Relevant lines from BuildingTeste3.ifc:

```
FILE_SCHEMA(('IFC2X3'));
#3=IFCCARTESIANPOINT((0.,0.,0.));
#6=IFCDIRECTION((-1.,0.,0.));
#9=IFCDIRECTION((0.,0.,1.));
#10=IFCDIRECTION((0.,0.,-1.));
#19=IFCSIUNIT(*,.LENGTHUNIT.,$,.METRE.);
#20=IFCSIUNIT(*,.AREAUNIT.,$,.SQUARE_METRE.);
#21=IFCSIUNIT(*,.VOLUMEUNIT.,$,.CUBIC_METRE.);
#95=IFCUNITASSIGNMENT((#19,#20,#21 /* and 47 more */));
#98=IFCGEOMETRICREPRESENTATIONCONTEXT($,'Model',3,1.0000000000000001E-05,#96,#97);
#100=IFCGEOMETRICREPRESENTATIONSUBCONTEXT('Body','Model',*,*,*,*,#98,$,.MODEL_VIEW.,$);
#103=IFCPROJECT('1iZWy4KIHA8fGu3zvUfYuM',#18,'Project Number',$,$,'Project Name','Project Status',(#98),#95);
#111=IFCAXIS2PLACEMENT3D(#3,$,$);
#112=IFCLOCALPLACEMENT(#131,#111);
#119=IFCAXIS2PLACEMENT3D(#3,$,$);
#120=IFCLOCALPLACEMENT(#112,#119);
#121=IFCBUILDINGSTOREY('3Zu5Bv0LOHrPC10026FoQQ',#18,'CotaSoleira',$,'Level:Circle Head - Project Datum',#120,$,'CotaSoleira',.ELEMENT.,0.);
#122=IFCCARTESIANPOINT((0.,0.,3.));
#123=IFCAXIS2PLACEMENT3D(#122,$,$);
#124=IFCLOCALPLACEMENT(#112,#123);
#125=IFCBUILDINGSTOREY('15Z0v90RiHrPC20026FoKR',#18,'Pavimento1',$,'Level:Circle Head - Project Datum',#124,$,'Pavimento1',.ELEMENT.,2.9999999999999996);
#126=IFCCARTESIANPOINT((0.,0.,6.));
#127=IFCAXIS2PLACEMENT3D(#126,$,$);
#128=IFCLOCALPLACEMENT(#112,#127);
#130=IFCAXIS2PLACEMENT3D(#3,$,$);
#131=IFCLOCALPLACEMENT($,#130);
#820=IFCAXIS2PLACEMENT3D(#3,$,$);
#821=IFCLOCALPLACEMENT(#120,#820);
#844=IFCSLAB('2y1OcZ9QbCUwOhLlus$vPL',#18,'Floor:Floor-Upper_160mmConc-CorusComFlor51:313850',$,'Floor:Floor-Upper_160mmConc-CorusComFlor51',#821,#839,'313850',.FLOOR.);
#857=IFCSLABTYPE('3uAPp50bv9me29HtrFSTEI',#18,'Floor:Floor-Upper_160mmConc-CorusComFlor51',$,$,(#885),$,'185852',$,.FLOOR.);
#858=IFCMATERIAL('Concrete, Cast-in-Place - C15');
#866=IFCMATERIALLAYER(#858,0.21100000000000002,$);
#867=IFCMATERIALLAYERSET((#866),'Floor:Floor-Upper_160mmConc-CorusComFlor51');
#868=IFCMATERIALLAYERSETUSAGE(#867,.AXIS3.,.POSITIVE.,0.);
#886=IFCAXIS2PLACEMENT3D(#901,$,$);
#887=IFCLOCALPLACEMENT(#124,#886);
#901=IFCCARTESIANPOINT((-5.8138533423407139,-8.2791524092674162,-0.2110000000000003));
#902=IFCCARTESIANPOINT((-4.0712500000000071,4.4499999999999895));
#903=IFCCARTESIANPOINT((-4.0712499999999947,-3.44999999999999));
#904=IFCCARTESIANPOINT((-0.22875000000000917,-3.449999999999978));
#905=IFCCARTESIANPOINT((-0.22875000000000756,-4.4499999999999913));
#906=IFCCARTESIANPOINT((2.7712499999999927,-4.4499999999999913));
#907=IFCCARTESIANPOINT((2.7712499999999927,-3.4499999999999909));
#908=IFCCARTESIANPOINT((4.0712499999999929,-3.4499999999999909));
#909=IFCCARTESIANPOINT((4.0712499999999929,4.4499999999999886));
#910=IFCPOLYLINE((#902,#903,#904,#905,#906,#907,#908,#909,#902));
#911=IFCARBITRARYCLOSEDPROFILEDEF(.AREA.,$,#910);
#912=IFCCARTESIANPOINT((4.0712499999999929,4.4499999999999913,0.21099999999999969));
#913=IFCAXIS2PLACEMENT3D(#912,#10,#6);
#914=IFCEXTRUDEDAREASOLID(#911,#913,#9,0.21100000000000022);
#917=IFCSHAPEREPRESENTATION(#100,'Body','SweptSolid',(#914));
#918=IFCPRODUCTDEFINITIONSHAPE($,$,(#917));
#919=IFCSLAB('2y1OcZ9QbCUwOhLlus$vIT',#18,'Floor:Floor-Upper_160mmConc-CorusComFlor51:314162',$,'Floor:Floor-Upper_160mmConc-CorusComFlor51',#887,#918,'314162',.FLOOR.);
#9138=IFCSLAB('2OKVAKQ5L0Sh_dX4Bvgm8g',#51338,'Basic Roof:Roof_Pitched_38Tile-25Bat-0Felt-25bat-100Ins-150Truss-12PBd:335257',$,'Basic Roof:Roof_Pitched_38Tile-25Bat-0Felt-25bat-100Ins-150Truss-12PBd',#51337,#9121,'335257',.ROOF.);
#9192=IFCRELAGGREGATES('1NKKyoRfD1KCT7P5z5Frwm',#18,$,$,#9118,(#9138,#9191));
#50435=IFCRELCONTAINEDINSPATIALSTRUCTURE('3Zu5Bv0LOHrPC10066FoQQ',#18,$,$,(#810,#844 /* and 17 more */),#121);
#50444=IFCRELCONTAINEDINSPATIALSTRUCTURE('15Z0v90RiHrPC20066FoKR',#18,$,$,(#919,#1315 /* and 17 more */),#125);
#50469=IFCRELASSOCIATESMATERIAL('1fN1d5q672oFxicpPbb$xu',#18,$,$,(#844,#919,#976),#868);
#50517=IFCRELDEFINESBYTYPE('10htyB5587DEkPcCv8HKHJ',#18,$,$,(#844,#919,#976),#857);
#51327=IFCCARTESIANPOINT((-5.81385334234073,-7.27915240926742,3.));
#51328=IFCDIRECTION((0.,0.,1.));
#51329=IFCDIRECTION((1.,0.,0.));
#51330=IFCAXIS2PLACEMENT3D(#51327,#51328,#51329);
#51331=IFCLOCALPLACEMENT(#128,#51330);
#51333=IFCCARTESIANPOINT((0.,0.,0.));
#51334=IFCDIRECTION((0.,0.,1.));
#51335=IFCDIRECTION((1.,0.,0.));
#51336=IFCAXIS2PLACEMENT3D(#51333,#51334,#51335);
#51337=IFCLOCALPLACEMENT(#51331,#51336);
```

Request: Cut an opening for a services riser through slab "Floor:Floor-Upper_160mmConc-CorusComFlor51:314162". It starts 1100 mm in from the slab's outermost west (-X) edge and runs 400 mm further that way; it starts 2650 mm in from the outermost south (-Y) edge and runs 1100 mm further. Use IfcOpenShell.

```python
import numpy as np
import ifcopenshell
import ifcopenshell.api.feature
import ifcopenshell.api.geometry
import ifcopenshell.api.root
import ifcopenshell.geom
import ifcopenshell.util.placement
import ifcopenshell.util.representation
import ifcopenshell.util.shape
import ifcopenshell.util.unit

model = ifcopenshell.open("BuildingTeste3.ifc")
unit_scale = ifcopenshell.util.unit.calculate_unit_scale(model)
settings = ifcopenshell.geom.settings()


def volume(element):
    """Net volume in cubic metres, openings subtracted."""
    shape = ifcopenshell.geom.create_shape(settings, element)
    return ifcopenshell.util.shape.get_volume(shape.geometry)


slab = model.by_guid("2y1OcZ9QbCUwOhLlus$vIT")
before = volume(slab)

# Extent in the slab's own axes, in metres. The edges named are its -X and -Y sides.
slab_shape = ifcopenshell.geom.create_shape(settings, slab)
vertices = ifcopenshell.util.shape.get_vertices(slab_shape.geometry)
x_min, y_min, bottom = vertices.min(axis=0)
top = vertices[:, 2].max()

opening = ifcopenshell.api.root.create_entity(model, ifc_class="IfcOpeningElement", name="Services riser opening")
context = ifcopenshell.util.representation.get_context(model, "Model", "Body", "MODEL_VIEW")
width, depth = 0.4, 1.1
outline = [(0.0, 0.0), (width, 0.0), (width, depth), (0.0, depth), (0.0, 0.0)]
# Overshoot both faces by 50 mm so the cut is clean.
shape = ifcopenshell.api.geometry.add_slab_representation(
    model, context=context, depth=top - bottom + 0.1, polyline=outline
)
ifcopenshell.api.geometry.assign_representation(model, product=opening, representation=shape)

matrix = ifcopenshell.util.placement.get_local_placement(slab.ObjectPlacement)
matrix[:, 3] = matrix @ np.append(np.array([x_min + 1.1, y_min + 2.65, bottom - 0.05]) / unit_scale, 1.0)
ifcopenshell.api.geometry.edit_object_placement(model, product=opening, matrix=matrix, is_si=False)
ifcopenshell.api.feature.add_feature(model, feature=opening, element=slab)

after = volume(slab)

print(f"slab volume {before:.3f} -> {after:.3f} m3")

model.write("BuildingTeste3-out.ifc")
```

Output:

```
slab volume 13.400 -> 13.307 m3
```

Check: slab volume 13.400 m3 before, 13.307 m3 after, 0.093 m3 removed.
